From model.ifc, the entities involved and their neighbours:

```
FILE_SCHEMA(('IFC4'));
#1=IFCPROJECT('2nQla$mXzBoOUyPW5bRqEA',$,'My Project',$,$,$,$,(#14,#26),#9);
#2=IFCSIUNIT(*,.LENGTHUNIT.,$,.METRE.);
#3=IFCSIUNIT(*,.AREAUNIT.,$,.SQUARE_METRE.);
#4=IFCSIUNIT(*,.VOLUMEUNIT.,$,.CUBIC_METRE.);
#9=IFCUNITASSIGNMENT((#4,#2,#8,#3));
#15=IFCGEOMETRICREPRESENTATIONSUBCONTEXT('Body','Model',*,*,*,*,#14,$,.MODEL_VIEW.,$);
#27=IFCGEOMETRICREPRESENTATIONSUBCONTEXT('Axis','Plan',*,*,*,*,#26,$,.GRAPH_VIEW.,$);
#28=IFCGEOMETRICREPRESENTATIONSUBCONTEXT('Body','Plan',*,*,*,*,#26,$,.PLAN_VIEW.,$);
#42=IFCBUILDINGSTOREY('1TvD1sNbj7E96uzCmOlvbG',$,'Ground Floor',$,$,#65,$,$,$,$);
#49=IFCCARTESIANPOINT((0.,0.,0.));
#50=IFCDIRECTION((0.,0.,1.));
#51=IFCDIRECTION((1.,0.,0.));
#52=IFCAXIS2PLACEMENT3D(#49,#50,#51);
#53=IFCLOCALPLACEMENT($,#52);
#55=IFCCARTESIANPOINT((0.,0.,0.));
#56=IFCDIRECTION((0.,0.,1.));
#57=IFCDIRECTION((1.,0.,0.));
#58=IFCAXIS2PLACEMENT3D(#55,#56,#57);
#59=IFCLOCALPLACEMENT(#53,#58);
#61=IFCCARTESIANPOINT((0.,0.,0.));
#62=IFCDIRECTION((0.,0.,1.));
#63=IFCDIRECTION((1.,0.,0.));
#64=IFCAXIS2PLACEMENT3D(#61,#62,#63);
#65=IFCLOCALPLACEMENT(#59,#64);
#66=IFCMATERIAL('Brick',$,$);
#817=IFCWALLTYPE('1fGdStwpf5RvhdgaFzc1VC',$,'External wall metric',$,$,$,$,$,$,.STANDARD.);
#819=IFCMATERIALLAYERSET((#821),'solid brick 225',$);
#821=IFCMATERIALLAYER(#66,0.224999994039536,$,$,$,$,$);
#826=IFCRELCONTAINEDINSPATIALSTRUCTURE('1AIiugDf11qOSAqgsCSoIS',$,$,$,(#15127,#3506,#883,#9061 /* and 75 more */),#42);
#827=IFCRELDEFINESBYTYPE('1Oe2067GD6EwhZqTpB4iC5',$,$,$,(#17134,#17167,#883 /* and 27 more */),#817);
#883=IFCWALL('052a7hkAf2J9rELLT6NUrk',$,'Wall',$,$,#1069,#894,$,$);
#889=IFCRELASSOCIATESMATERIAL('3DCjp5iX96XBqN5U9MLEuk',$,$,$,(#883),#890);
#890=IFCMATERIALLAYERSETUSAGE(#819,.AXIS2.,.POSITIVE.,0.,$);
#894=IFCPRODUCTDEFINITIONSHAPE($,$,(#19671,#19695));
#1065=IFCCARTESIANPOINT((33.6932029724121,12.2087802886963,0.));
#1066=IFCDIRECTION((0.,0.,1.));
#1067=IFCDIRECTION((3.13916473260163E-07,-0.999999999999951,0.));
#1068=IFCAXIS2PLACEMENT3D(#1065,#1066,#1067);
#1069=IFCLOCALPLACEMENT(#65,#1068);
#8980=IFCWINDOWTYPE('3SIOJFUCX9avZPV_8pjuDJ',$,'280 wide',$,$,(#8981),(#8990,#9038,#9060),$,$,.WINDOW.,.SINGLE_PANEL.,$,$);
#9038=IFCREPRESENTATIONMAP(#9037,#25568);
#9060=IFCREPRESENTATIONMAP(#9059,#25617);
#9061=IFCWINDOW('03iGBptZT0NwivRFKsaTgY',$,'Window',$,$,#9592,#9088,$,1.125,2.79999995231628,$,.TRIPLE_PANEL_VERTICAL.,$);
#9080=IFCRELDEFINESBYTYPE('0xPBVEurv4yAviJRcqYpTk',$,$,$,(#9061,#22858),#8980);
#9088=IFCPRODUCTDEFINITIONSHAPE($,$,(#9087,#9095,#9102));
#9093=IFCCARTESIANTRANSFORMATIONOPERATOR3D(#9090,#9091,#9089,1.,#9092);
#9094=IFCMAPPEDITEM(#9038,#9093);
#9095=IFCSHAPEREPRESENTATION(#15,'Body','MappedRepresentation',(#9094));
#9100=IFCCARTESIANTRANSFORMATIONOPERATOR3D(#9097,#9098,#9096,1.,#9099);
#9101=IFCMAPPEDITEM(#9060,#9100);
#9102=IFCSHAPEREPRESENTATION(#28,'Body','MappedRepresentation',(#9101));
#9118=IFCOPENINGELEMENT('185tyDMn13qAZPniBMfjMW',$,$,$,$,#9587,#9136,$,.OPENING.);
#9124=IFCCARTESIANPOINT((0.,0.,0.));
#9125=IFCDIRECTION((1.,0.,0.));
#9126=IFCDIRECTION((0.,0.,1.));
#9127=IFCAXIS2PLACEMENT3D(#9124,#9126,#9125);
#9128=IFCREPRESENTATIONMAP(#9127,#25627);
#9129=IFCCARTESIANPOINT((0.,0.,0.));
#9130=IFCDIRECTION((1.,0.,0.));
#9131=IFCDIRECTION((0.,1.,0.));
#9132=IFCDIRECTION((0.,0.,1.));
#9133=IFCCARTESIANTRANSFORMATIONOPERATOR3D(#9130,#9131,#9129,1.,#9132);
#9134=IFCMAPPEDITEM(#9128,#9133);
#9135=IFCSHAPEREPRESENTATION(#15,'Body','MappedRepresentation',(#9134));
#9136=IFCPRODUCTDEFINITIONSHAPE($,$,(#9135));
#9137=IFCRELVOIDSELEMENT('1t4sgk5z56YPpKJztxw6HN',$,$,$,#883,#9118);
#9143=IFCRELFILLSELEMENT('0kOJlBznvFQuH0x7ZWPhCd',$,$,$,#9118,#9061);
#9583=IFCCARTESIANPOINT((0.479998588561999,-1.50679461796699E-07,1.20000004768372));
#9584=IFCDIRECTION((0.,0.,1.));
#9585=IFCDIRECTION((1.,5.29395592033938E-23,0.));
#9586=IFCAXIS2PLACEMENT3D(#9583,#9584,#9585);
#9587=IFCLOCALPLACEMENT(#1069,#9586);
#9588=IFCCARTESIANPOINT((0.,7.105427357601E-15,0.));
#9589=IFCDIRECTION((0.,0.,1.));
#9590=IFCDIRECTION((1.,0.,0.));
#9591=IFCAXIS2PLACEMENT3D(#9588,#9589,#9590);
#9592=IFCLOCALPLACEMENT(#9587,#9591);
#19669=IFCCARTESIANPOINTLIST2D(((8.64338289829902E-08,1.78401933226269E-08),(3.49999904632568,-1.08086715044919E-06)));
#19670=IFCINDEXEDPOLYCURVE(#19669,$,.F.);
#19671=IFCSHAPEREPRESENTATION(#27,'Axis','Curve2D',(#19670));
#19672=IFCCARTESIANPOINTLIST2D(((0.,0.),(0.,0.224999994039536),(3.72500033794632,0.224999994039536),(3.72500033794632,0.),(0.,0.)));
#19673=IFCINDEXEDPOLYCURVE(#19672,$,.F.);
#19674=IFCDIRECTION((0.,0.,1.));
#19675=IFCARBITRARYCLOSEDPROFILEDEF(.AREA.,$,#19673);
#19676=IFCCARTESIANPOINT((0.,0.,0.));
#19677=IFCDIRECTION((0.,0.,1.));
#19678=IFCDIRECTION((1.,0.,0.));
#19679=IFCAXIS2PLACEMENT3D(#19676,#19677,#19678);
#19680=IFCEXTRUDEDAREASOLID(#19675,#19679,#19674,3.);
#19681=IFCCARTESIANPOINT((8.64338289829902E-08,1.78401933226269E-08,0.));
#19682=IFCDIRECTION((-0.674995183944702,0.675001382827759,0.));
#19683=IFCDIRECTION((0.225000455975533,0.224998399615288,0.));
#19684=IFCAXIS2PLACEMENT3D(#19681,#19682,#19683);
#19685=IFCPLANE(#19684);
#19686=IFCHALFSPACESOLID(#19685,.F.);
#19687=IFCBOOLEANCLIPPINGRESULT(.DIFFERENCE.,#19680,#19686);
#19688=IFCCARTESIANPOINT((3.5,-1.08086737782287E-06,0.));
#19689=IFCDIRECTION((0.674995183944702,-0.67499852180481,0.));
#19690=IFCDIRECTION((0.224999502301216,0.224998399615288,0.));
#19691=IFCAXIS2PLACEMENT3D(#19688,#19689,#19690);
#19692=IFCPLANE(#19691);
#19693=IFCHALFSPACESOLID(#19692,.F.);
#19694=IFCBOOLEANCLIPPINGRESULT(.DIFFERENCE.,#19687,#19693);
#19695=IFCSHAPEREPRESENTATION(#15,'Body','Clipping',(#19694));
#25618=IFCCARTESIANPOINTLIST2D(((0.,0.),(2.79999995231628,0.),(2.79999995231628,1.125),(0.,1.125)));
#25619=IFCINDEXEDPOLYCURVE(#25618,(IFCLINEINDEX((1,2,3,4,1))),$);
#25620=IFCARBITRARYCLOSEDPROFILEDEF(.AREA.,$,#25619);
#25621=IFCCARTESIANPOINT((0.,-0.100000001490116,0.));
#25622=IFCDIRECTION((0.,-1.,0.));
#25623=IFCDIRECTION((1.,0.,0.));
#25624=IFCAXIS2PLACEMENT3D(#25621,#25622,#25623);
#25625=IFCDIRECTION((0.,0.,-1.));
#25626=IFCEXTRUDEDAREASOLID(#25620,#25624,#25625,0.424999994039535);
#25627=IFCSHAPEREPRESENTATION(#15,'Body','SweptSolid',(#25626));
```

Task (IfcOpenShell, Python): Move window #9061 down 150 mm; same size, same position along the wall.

```python
import numpy as np
import ifcopenshell
import ifcopenshell.api.geometry
import ifcopenshell.util.placement
import ifcopenshell.util.unit

model = ifcopenshell.open("model.ifc")
unit_scale = ifcopenshell.util.unit.calculate_unit_scale(model)

window = model.by_guid("03iGBptZT0NwivRFKsaTgY")
opening = window.FillsVoids[0].RelatingOpeningElement
dz = -0.15 / unit_scale

shift = np.array([0.0, 0.0, dz])
# The window is placed relative to its opening, so it follows when the opening moves.
matrix = ifcopenshell.util.placement.get_local_placement(opening.ObjectPlacement)
matrix[:3, 3] += shift
ifcopenshell.api.geometry.edit_object_placement(
    model, product=opening, matrix=matrix, is_si=False, should_transform_children=True
)

print(f"moved by {dz * unit_scale:+.3f} m")

model.write("model_v2.ifc")
```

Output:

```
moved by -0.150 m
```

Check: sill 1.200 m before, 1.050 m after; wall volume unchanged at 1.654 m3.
